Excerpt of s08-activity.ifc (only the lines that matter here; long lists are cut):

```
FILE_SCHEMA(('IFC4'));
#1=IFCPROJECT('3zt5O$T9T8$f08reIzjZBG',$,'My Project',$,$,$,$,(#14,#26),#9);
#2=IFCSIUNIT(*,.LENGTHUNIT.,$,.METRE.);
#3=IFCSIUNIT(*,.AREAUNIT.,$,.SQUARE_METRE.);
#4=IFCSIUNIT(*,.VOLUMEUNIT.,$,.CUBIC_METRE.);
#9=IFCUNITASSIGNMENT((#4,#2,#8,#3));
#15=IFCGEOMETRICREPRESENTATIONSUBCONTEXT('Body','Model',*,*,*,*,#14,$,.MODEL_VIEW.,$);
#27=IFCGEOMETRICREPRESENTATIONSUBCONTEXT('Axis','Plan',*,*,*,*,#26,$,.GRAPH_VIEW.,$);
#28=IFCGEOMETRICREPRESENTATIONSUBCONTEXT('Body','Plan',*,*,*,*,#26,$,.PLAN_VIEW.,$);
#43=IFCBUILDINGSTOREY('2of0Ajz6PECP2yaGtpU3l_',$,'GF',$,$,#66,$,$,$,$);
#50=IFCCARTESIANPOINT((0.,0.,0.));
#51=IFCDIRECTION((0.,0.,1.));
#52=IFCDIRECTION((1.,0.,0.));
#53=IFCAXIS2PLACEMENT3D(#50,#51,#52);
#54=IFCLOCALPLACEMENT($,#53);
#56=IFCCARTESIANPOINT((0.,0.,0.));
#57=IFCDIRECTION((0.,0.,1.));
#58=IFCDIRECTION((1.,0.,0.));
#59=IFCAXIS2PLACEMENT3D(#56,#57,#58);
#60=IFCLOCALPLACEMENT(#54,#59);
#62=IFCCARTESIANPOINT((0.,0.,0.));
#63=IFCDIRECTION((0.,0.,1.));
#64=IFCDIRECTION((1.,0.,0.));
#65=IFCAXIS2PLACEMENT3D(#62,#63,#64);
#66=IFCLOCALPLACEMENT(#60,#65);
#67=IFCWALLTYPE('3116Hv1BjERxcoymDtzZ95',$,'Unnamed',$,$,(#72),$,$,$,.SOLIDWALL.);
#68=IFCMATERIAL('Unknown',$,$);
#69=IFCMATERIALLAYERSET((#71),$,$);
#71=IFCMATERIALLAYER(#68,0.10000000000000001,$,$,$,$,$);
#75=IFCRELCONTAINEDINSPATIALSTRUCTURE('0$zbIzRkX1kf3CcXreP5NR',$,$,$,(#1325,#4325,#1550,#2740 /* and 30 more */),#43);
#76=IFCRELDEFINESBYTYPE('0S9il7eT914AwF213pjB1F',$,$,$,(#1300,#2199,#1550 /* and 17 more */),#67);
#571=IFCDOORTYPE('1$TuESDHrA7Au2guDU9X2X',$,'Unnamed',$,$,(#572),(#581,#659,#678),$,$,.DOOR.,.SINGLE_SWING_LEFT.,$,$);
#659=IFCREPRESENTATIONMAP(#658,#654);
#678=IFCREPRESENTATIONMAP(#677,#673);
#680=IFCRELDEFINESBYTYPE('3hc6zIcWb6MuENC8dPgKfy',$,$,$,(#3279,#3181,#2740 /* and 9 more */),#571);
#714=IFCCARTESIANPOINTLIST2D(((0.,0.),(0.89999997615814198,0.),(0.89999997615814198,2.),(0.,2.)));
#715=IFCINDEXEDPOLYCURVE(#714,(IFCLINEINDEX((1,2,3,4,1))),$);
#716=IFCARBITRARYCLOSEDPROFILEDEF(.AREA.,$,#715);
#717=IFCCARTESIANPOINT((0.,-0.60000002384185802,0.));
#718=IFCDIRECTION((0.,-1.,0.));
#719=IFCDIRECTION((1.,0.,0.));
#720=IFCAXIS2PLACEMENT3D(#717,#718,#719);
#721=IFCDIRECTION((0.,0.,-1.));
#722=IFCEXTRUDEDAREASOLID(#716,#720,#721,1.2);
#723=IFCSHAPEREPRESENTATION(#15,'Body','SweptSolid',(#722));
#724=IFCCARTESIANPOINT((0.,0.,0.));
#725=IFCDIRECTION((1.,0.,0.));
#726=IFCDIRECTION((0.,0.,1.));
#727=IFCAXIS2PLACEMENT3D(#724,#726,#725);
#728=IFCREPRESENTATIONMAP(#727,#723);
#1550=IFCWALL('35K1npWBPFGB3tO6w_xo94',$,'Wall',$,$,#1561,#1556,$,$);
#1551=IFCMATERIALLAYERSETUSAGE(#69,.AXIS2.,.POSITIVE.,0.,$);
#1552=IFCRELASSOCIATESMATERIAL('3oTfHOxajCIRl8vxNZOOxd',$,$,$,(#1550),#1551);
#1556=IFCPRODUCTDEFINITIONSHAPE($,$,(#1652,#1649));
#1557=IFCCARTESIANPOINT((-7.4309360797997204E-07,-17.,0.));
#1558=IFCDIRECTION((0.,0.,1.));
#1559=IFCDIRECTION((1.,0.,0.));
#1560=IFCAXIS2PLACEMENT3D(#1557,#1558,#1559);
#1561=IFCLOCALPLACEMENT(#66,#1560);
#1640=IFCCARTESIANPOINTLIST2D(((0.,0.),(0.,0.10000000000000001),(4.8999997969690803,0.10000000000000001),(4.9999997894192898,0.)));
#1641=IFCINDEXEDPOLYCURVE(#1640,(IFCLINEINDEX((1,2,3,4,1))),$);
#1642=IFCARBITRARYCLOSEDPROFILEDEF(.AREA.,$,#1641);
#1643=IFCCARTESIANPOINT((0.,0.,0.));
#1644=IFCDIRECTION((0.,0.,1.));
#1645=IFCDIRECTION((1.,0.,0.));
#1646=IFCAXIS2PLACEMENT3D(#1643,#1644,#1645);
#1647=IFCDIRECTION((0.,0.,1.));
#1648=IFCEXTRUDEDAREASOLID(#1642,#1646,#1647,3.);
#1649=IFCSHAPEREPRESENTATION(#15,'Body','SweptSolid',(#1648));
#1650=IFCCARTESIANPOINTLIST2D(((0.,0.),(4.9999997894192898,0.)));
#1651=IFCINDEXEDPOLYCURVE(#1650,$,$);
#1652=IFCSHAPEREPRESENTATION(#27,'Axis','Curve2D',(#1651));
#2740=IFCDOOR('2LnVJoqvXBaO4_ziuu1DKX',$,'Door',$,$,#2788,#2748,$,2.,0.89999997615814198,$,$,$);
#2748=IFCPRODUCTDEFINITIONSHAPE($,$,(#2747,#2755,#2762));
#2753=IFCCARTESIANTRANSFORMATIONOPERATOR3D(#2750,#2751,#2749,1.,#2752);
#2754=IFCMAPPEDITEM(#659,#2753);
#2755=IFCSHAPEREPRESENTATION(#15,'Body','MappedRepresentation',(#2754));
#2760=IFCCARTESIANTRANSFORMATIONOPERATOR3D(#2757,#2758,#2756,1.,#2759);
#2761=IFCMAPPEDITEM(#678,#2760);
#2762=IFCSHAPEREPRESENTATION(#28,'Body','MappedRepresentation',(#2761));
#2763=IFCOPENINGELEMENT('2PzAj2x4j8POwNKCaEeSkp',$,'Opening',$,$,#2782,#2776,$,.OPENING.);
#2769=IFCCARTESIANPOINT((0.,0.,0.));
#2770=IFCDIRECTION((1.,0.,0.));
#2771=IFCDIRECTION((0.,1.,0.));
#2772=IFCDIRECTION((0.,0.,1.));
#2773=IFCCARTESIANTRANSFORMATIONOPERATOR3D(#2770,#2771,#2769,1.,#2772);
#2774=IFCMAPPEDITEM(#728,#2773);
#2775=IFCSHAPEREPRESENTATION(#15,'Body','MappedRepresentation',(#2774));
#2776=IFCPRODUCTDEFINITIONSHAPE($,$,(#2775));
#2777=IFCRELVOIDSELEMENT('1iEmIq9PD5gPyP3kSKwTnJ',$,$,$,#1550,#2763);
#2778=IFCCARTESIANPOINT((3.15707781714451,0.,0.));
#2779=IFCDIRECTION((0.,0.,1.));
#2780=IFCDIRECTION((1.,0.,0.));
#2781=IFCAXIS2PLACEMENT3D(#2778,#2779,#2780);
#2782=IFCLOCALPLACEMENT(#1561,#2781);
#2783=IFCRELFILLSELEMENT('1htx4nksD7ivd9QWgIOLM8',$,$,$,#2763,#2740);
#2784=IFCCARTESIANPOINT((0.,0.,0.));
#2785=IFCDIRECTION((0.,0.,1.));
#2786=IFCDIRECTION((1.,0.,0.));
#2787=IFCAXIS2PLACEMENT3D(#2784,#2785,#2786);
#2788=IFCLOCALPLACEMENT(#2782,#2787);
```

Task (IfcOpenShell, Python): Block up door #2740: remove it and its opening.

```python
import ifcopenshell
import ifcopenshell.api.feature
import ifcopenshell.api.root
import ifcopenshell.geom
import ifcopenshell.util.shape

model = ifcopenshell.open("s08-activity.ifc")
settings = ifcopenshell.geom.settings()


def volume(element):
    """Net volume in cubic metres, openings subtracted."""
    shape = ifcopenshell.geom.create_shape(settings, element)
    return ifcopenshell.util.shape.get_volume(shape.geometry)


door = model.by_guid("2LnVJoqvXBaO4_ziuu1DKX")
opening = door.FillsVoids[0].RelatingOpeningElement
wall = opening.VoidsElements[0].RelatingBuildingElement
before = volume(wall)

ifcopenshell.api.root.remove_product(model, product=door)
ifcopenshell.api.feature.remove_feature(model, feature=opening)

after = volume(wall)

print(f"wall volume {before:.3f} -> {after:.3f} m3")

model.write("s08-activity_updated.ifc")
```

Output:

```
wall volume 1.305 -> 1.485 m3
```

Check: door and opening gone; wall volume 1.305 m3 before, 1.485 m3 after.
